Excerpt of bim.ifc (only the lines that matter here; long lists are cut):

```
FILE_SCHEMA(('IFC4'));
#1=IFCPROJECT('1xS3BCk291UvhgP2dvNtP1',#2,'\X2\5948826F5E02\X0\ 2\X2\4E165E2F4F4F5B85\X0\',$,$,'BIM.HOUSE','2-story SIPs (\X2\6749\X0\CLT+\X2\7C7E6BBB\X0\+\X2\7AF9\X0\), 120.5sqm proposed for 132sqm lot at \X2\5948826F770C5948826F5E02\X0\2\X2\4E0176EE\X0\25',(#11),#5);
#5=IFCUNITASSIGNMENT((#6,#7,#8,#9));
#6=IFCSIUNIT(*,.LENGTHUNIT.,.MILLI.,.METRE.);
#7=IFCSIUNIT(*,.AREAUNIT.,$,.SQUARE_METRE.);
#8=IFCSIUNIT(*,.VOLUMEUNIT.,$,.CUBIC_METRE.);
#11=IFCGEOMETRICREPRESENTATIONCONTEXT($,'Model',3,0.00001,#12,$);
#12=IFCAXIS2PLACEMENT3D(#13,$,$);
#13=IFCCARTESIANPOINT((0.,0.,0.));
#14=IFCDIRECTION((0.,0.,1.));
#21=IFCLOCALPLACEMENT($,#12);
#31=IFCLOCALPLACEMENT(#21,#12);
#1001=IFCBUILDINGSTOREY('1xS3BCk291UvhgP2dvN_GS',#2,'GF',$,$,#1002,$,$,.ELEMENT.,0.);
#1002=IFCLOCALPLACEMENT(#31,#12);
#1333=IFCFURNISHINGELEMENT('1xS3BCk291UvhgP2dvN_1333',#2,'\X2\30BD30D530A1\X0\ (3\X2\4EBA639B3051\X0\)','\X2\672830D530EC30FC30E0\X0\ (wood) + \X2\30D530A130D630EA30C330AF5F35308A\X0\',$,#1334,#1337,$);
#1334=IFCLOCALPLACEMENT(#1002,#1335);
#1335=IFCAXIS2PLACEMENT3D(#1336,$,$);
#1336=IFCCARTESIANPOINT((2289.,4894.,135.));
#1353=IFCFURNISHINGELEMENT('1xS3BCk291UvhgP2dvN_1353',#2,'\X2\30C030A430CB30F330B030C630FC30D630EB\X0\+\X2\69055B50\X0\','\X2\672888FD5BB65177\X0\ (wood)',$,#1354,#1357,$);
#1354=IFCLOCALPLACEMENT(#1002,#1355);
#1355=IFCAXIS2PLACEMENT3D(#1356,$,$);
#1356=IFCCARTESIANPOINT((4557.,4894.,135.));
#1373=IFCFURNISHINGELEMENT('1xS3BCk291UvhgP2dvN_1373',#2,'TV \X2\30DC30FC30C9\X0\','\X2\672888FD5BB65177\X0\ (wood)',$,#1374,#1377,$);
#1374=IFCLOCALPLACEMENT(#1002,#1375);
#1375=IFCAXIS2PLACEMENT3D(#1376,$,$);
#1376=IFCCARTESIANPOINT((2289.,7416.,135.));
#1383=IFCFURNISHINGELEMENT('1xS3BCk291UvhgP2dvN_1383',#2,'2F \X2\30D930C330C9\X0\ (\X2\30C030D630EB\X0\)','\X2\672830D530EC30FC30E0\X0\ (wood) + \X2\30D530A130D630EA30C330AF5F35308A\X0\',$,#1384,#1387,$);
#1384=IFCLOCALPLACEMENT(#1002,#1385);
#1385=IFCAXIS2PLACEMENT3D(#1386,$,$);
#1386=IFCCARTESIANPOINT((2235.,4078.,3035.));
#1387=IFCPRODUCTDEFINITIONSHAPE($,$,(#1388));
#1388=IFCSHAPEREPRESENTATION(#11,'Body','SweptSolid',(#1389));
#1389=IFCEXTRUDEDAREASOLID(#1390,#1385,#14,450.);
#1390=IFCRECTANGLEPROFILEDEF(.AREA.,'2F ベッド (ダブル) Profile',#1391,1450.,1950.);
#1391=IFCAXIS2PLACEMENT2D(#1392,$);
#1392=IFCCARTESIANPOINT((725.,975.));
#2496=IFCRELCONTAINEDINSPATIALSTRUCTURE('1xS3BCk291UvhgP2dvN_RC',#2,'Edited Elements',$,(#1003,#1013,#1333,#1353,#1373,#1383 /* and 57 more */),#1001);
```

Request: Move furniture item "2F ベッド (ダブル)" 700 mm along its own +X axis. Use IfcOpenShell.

```python
import ifcopenshell
import ifcopenshell.api.geometry
import ifcopenshell.util.placement
import ifcopenshell.util.unit

model = ifcopenshell.open("bim.ifc")
unit_scale = ifcopenshell.util.unit.calculate_unit_scale(model)

item = model.by_id(1383)
matrix = ifcopenshell.util.placement.get_local_placement(item.ObjectPlacement)
matrix[:3, 3] += matrix[:3, 0] * 0.7 / unit_scale
ifcopenshell.api.geometry.edit_object_placement(model, product=item, matrix=matrix, is_si=False)

print(ifcopenshell.util.placement.get_local_placement(item.ObjectPlacement).round(3) + 0.0)

model.write("bim-out.ifc")
```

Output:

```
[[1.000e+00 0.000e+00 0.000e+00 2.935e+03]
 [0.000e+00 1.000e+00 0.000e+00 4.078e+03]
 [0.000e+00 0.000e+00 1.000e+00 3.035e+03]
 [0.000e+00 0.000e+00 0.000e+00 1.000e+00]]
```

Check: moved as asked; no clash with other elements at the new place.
